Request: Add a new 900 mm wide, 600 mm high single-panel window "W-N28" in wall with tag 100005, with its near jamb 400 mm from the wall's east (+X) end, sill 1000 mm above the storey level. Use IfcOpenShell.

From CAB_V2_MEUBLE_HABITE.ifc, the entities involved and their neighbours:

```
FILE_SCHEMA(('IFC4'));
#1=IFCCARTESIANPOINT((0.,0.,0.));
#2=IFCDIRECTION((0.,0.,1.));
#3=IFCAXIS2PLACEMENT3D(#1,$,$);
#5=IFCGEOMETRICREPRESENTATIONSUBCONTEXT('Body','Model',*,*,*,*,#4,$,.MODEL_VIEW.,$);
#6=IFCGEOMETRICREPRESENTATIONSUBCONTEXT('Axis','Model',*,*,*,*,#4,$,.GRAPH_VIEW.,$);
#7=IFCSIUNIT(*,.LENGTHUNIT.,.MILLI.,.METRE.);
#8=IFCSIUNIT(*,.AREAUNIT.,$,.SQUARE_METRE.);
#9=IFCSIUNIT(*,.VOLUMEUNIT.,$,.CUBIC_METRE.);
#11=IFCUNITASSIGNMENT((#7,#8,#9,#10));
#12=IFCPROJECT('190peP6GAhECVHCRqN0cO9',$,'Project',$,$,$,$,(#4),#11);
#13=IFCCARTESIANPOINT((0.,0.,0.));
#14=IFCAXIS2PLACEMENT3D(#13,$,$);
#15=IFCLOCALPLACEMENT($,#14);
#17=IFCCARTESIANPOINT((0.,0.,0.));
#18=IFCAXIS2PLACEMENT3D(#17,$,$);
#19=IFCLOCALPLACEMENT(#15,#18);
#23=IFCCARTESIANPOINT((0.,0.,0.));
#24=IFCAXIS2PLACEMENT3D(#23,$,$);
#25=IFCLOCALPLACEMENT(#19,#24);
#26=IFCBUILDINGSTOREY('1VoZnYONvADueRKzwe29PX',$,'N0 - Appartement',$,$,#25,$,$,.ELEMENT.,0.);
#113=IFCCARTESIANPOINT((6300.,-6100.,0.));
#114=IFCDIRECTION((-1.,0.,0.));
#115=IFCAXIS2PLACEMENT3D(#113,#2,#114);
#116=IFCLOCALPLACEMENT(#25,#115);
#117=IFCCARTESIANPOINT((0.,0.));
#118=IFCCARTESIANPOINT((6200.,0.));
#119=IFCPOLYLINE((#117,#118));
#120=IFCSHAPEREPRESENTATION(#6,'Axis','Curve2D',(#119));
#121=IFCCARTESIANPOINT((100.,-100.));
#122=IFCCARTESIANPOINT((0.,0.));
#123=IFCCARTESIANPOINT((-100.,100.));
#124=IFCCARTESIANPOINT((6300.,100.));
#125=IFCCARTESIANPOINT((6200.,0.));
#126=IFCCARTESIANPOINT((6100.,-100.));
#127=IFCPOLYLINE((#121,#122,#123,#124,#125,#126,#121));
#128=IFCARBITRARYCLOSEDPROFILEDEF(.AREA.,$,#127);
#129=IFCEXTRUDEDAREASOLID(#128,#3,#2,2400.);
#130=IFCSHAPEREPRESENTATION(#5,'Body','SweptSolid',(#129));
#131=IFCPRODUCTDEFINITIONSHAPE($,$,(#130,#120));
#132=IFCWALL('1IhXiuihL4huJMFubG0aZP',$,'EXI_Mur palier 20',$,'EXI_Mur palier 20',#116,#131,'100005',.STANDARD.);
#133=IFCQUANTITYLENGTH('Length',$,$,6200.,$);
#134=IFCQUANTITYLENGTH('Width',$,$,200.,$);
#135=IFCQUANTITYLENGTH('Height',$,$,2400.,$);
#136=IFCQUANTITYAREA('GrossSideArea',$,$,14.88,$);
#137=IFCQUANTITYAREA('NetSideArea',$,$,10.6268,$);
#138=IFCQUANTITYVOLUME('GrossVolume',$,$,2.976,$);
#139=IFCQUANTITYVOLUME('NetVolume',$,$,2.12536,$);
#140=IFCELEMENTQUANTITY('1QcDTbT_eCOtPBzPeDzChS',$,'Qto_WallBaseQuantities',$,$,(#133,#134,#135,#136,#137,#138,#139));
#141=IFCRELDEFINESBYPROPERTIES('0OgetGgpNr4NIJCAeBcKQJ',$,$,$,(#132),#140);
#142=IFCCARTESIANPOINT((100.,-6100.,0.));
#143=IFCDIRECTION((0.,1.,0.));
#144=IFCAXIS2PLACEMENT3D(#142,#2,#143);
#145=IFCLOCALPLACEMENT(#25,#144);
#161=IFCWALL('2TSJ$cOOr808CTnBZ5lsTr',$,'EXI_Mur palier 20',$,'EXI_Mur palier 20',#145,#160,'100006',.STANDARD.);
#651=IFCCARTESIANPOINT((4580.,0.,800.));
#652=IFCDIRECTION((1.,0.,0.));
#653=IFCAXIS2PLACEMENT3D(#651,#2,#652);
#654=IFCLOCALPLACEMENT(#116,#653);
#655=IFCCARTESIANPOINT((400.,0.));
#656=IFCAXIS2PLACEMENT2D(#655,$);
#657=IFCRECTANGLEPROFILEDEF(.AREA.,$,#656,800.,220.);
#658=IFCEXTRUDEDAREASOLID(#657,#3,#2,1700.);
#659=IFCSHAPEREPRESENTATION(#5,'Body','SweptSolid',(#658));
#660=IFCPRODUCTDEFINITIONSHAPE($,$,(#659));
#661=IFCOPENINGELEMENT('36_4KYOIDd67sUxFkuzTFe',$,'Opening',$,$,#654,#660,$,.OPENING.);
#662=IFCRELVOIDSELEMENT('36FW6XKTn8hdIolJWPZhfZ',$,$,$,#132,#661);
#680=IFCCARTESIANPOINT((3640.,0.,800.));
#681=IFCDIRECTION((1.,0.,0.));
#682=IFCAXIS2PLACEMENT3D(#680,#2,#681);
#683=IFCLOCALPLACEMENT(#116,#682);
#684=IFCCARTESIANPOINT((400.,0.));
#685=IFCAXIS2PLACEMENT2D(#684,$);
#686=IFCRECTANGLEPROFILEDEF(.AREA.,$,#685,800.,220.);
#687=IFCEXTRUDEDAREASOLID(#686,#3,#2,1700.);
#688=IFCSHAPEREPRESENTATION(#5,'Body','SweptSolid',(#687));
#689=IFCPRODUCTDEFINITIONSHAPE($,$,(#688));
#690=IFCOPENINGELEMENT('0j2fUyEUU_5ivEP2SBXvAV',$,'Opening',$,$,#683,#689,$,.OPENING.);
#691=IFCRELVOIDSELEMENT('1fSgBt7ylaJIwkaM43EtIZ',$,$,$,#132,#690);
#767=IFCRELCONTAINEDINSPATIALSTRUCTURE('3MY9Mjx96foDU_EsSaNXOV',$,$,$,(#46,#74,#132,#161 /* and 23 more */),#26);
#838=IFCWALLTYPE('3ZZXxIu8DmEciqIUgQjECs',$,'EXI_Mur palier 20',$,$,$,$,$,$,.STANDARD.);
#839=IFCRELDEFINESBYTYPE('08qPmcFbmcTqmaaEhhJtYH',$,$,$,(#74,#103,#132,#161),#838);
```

```python
import numpy as np
import ifcopenshell
import ifcopenshell.api.feature
import ifcopenshell.api.geometry
import ifcopenshell.api.pset
import ifcopenshell.api.root
import ifcopenshell.api.spatial
import ifcopenshell.geom
import ifcopenshell.util.element
import ifcopenshell.util.placement
import ifcopenshell.util.representation
import ifcopenshell.util.shape
import ifcopenshell.util.unit

model = ifcopenshell.open("CAB_V2_MEUBLE_HABITE.ifc")
unit_scale = ifcopenshell.util.unit.calculate_unit_scale(model)
area_scale = ifcopenshell.util.unit.calculate_unit_scale(model, "AREAUNIT")
volume_scale = ifcopenshell.util.unit.calculate_unit_scale(model, "VOLUMEUNIT")
settings = ifcopenshell.geom.settings()


def volume(element):
    """Net volume in cubic metres, openings subtracted."""
    shape = ifcopenshell.geom.create_shape(settings, element)
    return ifcopenshell.util.shape.get_volume(shape.geometry)


wall = model.by_guid("1IhXiuihL4huJMFubG0aZP")
storey = ifcopenshell.util.element.get_container(wall, ifc_class="IfcBuildingStorey")
context = ifcopenshell.util.representation.get_context(model, "Model", "Body", "MODEL_VIEW")
before = volume(wall)

width, height, from_end, sill = 0.9, 0.6, 0.4, 1  # metres

# The wall runs along its own X axis, and the end named is its -X end.
wall_shape = ifcopenshell.geom.create_shape(settings, wall)
x, y, z = ifcopenshell.util.shape.get_vertices(wall_shape.geometry).T
start = x.min() + from_end
face, thickness = float(y.min()), float(y.max() - y.min())
wall_matrix = ifcopenshell.util.placement.get_local_placement(wall.ObjectPlacement)
level = ifcopenshell.util.placement.get_local_placement(storey.ObjectPlacement)[2, 3]


def in_wall(x, y):
    """Placement at x, y metres in the wall's axes, at sill height."""
    matrix = wall_matrix.copy()
    matrix[:, 3] = wall_matrix @ np.array([x / unit_scale, y / unit_scale, 0.0, 1.0])
    matrix[2, 3] = level + sill / unit_scale
    return matrix


# Opening: a box that overshoots both wall faces by 50 mm.
opening = ifcopenshell.api.root.create_entity(model, ifc_class="IfcOpeningElement", predefined_type="OPENING")
box = ifcopenshell.api.geometry.add_wall_representation(
    model, context=context, length=width, height=height, thickness=thickness + 0.1
)
ifcopenshell.api.geometry.assign_representation(model, product=opening, representation=box)
ifcopenshell.api.geometry.edit_object_placement(model, product=opening, matrix=in_wall(start, face - 0.05), is_si=False)
ifcopenshell.api.feature.add_feature(model, feature=opening, element=wall)

window = ifcopenshell.api.root.create_entity(model, ifc_class="IfcWindow", name="W-N28", predefined_type="WINDOW")
window.OverallWidth, window.OverallHeight = width / unit_scale, height / unit_scale
window.PartitioningType = "SINGLE_PANEL"
body = ifcopenshell.api.geometry.add_window_representation(
    model,
    context=context,
    overall_width=window.OverallWidth,
    overall_height=window.OverallHeight,
    partition_type="SINGLE_PANEL",
)
ifcopenshell.api.geometry.assign_representation(model, product=window, representation=body)
ifcopenshell.api.spatial.assign_container(model, products=[window], relating_structure=storey)
ifcopenshell.api.feature.add_filling(model, opening=opening, element=window)

# Centre the window in the wall's thickness.
ifcopenshell.api.geometry.edit_object_placement(model, product=window, matrix=in_wall(start, face), is_si=False)
window_shape = ifcopenshell.geom.create_shape(settings, window)
depth = ifcopenshell.util.shape.get_vertices(window_shape.geometry)[:, 1]
offset = face + thickness / 2 - (depth.min() + depth.max()) / 2
ifcopenshell.api.geometry.edit_object_placement(model, product=window, matrix=in_wall(start, offset), is_si=False)

after = volume(wall)

# Update the wall's stored quantities.
qto = model.by_id(ifcopenshell.util.element.get_pset(wall, "Qto_WallBaseQuantities", should_inherit=False)["id"])
ifcopenshell.api.pset.edit_qto(model, qto=qto, properties={
    "NetSideArea": after / thickness / area_scale,
    "NetVolume": after / volume_scale,
})

print(f"wall volume {before:.3f} -> {after:.3f} m3")

model.write("CAB_V2_MEUBLE_HABITE_edited.ifc")
```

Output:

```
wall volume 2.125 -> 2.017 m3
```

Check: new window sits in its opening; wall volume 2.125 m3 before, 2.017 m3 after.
